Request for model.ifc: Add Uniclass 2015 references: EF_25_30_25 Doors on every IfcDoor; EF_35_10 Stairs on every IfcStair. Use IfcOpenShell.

First a look at what the model holds.

```python
import ifcopenshell

model = ifcopenshell.open("model.ifc")
print(model.schema)
print("classifications:", [c.Name for c in model.by_type("IfcClassification")])
for ifc_class in ("IfcDoor", "IfcRoof", "IfcStair", "IfcWall", "IfcWindow"):
    print(ifc_class, len(model.by_type(ifc_class)))
```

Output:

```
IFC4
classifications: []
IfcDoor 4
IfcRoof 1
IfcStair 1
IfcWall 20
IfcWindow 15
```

```python
import ifcopenshell
import ifcopenshell.api.classification

model = ifcopenshell.open("model.ifc")

system = ifcopenshell.api.classification.add_classification(model, classification="Uniclass 2015")

codes = {
    "IfcDoor": ("EF_25_30_25", "Doors"),
    "IfcStair": ("EF_35_10", "Stairs"),
}
for ifc_class, (code, name) in codes.items():
    products = model.by_type(ifc_class)
    ifcopenshell.api.classification.add_reference(
        model, products=products, classification=system, identification=code, name=name
    )
    print(code, len(products))

model.write("model-out.ifc")
```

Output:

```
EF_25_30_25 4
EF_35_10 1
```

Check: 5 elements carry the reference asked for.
